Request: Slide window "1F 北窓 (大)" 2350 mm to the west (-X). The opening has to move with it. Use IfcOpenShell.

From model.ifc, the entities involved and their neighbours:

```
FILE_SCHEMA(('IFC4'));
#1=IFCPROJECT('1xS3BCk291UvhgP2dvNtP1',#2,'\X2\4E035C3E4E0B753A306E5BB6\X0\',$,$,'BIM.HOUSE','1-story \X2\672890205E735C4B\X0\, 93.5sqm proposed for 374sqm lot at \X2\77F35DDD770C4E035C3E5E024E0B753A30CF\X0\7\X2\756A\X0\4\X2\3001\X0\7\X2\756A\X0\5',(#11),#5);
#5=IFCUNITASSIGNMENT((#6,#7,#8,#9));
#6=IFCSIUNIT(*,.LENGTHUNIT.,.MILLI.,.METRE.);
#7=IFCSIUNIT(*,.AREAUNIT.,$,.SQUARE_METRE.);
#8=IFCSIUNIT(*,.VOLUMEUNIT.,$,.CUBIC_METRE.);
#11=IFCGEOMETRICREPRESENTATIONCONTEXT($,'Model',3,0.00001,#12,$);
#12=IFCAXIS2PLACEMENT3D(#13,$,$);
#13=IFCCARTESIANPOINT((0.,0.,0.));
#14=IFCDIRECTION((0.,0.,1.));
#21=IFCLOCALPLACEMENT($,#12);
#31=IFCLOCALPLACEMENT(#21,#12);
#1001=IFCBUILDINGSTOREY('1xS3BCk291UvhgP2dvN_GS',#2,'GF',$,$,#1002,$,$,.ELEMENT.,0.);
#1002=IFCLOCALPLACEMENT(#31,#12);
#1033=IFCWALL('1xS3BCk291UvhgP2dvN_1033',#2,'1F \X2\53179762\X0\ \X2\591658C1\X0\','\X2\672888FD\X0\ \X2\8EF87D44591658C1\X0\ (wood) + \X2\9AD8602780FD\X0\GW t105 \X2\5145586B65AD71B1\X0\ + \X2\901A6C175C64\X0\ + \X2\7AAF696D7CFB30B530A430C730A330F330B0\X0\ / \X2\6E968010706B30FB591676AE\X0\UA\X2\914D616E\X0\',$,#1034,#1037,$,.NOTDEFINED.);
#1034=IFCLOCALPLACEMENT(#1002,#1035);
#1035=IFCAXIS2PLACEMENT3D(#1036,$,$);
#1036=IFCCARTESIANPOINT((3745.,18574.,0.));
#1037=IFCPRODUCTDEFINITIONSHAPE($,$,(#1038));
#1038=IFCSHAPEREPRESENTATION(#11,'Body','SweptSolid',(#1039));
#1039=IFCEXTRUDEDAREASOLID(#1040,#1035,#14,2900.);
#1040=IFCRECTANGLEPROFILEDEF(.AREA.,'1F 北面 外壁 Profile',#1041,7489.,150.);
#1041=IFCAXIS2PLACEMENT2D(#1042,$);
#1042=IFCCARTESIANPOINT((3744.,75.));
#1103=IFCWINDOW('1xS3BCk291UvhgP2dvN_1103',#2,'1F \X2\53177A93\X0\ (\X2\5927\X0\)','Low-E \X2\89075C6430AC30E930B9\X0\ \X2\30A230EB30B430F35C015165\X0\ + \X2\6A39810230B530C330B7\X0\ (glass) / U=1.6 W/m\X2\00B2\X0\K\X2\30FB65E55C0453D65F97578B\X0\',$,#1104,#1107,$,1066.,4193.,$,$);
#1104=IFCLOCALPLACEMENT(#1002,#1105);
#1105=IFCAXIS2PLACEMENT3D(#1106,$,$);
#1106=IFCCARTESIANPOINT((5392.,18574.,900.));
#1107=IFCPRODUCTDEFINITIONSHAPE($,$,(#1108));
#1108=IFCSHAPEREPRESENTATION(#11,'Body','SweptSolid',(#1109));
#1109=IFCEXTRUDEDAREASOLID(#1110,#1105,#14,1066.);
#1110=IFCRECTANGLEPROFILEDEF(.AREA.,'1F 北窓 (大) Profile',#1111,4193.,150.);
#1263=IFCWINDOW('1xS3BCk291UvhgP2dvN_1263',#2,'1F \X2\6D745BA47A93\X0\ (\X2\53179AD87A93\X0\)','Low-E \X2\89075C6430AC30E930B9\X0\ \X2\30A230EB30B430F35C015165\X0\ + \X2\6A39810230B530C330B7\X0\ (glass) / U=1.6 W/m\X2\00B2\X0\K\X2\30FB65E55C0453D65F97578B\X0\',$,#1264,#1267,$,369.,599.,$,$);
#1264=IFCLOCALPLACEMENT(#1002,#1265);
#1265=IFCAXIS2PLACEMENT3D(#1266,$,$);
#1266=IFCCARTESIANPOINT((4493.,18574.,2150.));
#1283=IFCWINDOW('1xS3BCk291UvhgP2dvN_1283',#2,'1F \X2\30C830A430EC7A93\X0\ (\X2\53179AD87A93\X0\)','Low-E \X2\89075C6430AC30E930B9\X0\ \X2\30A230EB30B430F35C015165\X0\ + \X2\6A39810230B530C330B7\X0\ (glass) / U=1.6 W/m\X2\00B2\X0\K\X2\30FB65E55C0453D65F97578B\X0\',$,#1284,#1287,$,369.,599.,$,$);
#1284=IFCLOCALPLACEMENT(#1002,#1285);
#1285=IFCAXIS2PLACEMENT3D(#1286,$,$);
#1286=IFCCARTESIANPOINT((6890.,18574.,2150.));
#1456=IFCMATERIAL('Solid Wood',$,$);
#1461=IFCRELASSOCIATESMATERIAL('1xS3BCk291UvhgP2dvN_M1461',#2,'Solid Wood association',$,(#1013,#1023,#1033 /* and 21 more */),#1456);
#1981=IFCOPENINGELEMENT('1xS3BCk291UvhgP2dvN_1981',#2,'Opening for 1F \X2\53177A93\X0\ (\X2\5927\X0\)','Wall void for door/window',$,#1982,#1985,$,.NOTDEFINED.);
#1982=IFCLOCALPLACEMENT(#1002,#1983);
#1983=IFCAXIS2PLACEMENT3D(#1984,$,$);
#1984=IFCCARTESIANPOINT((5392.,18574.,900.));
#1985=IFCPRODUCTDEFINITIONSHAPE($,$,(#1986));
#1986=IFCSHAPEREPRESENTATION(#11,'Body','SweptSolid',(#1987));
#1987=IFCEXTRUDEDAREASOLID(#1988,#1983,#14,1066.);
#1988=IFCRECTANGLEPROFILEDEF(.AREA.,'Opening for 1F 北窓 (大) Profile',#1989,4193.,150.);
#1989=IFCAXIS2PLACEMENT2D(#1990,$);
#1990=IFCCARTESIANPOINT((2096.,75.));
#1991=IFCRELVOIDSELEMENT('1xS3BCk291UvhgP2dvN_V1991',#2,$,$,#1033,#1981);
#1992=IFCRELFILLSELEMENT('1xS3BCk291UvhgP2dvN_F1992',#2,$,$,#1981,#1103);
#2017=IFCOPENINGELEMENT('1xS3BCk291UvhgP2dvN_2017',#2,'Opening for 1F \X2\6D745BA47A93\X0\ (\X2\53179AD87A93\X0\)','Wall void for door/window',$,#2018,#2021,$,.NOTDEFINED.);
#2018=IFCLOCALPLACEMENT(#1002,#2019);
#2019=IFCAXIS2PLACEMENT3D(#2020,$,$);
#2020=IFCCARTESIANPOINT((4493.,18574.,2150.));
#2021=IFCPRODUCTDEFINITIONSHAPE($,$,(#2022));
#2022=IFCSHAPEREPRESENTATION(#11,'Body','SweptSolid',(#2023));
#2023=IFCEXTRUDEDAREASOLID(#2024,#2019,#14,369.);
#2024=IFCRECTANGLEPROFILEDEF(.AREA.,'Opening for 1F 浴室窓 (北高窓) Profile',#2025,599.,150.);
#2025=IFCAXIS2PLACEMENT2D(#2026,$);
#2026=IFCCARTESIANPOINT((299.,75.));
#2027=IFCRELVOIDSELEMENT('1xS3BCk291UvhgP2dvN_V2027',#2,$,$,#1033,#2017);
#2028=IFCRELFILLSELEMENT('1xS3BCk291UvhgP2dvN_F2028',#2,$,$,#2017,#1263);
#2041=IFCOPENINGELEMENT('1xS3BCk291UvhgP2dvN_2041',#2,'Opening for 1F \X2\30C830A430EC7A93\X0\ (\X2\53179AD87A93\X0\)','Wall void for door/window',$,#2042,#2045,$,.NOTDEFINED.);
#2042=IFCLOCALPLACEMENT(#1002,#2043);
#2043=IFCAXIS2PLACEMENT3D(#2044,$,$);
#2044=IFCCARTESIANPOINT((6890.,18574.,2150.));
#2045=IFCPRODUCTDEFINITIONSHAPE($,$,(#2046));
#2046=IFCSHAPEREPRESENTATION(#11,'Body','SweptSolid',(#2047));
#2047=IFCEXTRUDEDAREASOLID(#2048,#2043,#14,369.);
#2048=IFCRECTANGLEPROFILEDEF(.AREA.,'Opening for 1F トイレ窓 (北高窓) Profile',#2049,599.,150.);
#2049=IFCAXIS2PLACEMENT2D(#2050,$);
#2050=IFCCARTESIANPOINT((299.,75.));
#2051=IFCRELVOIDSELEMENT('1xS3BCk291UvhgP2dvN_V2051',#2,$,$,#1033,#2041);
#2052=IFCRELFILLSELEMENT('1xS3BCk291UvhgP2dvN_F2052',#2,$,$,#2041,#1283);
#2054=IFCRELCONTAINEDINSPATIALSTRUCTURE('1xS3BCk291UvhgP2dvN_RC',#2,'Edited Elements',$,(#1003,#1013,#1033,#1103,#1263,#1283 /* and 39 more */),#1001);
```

```python
import ifcopenshell
import ifcopenshell.api.geometry
import ifcopenshell.util.placement
import ifcopenshell.util.unit

model = ifcopenshell.open("model.ifc")
unit_scale = ifcopenshell.util.unit.calculate_unit_scale(model)

window = model.by_guid("1xS3BCk291UvhgP2dvN_1103")
opening = window.FillsVoids[0].RelatingOpeningElement
wall = opening.VoidsElements[0].RelatingBuildingElement

wall_matrix = ifcopenshell.util.placement.get_local_placement(wall.ObjectPlacement)
shift = wall_matrix[:3, 0] * -2.35 / unit_scale
before = ifcopenshell.util.placement.get_local_placement(window.ObjectPlacement)[:3, 3].copy()

# The window is not placed relative to its opening, so move both.
for product in (opening, window):
    matrix = ifcopenshell.util.placement.get_local_placement(product.ObjectPlacement)
    matrix[:3, 3] += shift
    ifcopenshell.api.geometry.edit_object_placement(model, product=product, matrix=matrix, is_si=False)

after = ifcopenshell.util.placement.get_local_placement(window.ObjectPlacement)[:3, 3]
print("window moved by", (after - before).round(3) + 0.0)

model.write("model-out.ifc")
```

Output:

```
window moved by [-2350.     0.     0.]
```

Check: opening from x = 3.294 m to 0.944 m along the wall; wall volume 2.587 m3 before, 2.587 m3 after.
